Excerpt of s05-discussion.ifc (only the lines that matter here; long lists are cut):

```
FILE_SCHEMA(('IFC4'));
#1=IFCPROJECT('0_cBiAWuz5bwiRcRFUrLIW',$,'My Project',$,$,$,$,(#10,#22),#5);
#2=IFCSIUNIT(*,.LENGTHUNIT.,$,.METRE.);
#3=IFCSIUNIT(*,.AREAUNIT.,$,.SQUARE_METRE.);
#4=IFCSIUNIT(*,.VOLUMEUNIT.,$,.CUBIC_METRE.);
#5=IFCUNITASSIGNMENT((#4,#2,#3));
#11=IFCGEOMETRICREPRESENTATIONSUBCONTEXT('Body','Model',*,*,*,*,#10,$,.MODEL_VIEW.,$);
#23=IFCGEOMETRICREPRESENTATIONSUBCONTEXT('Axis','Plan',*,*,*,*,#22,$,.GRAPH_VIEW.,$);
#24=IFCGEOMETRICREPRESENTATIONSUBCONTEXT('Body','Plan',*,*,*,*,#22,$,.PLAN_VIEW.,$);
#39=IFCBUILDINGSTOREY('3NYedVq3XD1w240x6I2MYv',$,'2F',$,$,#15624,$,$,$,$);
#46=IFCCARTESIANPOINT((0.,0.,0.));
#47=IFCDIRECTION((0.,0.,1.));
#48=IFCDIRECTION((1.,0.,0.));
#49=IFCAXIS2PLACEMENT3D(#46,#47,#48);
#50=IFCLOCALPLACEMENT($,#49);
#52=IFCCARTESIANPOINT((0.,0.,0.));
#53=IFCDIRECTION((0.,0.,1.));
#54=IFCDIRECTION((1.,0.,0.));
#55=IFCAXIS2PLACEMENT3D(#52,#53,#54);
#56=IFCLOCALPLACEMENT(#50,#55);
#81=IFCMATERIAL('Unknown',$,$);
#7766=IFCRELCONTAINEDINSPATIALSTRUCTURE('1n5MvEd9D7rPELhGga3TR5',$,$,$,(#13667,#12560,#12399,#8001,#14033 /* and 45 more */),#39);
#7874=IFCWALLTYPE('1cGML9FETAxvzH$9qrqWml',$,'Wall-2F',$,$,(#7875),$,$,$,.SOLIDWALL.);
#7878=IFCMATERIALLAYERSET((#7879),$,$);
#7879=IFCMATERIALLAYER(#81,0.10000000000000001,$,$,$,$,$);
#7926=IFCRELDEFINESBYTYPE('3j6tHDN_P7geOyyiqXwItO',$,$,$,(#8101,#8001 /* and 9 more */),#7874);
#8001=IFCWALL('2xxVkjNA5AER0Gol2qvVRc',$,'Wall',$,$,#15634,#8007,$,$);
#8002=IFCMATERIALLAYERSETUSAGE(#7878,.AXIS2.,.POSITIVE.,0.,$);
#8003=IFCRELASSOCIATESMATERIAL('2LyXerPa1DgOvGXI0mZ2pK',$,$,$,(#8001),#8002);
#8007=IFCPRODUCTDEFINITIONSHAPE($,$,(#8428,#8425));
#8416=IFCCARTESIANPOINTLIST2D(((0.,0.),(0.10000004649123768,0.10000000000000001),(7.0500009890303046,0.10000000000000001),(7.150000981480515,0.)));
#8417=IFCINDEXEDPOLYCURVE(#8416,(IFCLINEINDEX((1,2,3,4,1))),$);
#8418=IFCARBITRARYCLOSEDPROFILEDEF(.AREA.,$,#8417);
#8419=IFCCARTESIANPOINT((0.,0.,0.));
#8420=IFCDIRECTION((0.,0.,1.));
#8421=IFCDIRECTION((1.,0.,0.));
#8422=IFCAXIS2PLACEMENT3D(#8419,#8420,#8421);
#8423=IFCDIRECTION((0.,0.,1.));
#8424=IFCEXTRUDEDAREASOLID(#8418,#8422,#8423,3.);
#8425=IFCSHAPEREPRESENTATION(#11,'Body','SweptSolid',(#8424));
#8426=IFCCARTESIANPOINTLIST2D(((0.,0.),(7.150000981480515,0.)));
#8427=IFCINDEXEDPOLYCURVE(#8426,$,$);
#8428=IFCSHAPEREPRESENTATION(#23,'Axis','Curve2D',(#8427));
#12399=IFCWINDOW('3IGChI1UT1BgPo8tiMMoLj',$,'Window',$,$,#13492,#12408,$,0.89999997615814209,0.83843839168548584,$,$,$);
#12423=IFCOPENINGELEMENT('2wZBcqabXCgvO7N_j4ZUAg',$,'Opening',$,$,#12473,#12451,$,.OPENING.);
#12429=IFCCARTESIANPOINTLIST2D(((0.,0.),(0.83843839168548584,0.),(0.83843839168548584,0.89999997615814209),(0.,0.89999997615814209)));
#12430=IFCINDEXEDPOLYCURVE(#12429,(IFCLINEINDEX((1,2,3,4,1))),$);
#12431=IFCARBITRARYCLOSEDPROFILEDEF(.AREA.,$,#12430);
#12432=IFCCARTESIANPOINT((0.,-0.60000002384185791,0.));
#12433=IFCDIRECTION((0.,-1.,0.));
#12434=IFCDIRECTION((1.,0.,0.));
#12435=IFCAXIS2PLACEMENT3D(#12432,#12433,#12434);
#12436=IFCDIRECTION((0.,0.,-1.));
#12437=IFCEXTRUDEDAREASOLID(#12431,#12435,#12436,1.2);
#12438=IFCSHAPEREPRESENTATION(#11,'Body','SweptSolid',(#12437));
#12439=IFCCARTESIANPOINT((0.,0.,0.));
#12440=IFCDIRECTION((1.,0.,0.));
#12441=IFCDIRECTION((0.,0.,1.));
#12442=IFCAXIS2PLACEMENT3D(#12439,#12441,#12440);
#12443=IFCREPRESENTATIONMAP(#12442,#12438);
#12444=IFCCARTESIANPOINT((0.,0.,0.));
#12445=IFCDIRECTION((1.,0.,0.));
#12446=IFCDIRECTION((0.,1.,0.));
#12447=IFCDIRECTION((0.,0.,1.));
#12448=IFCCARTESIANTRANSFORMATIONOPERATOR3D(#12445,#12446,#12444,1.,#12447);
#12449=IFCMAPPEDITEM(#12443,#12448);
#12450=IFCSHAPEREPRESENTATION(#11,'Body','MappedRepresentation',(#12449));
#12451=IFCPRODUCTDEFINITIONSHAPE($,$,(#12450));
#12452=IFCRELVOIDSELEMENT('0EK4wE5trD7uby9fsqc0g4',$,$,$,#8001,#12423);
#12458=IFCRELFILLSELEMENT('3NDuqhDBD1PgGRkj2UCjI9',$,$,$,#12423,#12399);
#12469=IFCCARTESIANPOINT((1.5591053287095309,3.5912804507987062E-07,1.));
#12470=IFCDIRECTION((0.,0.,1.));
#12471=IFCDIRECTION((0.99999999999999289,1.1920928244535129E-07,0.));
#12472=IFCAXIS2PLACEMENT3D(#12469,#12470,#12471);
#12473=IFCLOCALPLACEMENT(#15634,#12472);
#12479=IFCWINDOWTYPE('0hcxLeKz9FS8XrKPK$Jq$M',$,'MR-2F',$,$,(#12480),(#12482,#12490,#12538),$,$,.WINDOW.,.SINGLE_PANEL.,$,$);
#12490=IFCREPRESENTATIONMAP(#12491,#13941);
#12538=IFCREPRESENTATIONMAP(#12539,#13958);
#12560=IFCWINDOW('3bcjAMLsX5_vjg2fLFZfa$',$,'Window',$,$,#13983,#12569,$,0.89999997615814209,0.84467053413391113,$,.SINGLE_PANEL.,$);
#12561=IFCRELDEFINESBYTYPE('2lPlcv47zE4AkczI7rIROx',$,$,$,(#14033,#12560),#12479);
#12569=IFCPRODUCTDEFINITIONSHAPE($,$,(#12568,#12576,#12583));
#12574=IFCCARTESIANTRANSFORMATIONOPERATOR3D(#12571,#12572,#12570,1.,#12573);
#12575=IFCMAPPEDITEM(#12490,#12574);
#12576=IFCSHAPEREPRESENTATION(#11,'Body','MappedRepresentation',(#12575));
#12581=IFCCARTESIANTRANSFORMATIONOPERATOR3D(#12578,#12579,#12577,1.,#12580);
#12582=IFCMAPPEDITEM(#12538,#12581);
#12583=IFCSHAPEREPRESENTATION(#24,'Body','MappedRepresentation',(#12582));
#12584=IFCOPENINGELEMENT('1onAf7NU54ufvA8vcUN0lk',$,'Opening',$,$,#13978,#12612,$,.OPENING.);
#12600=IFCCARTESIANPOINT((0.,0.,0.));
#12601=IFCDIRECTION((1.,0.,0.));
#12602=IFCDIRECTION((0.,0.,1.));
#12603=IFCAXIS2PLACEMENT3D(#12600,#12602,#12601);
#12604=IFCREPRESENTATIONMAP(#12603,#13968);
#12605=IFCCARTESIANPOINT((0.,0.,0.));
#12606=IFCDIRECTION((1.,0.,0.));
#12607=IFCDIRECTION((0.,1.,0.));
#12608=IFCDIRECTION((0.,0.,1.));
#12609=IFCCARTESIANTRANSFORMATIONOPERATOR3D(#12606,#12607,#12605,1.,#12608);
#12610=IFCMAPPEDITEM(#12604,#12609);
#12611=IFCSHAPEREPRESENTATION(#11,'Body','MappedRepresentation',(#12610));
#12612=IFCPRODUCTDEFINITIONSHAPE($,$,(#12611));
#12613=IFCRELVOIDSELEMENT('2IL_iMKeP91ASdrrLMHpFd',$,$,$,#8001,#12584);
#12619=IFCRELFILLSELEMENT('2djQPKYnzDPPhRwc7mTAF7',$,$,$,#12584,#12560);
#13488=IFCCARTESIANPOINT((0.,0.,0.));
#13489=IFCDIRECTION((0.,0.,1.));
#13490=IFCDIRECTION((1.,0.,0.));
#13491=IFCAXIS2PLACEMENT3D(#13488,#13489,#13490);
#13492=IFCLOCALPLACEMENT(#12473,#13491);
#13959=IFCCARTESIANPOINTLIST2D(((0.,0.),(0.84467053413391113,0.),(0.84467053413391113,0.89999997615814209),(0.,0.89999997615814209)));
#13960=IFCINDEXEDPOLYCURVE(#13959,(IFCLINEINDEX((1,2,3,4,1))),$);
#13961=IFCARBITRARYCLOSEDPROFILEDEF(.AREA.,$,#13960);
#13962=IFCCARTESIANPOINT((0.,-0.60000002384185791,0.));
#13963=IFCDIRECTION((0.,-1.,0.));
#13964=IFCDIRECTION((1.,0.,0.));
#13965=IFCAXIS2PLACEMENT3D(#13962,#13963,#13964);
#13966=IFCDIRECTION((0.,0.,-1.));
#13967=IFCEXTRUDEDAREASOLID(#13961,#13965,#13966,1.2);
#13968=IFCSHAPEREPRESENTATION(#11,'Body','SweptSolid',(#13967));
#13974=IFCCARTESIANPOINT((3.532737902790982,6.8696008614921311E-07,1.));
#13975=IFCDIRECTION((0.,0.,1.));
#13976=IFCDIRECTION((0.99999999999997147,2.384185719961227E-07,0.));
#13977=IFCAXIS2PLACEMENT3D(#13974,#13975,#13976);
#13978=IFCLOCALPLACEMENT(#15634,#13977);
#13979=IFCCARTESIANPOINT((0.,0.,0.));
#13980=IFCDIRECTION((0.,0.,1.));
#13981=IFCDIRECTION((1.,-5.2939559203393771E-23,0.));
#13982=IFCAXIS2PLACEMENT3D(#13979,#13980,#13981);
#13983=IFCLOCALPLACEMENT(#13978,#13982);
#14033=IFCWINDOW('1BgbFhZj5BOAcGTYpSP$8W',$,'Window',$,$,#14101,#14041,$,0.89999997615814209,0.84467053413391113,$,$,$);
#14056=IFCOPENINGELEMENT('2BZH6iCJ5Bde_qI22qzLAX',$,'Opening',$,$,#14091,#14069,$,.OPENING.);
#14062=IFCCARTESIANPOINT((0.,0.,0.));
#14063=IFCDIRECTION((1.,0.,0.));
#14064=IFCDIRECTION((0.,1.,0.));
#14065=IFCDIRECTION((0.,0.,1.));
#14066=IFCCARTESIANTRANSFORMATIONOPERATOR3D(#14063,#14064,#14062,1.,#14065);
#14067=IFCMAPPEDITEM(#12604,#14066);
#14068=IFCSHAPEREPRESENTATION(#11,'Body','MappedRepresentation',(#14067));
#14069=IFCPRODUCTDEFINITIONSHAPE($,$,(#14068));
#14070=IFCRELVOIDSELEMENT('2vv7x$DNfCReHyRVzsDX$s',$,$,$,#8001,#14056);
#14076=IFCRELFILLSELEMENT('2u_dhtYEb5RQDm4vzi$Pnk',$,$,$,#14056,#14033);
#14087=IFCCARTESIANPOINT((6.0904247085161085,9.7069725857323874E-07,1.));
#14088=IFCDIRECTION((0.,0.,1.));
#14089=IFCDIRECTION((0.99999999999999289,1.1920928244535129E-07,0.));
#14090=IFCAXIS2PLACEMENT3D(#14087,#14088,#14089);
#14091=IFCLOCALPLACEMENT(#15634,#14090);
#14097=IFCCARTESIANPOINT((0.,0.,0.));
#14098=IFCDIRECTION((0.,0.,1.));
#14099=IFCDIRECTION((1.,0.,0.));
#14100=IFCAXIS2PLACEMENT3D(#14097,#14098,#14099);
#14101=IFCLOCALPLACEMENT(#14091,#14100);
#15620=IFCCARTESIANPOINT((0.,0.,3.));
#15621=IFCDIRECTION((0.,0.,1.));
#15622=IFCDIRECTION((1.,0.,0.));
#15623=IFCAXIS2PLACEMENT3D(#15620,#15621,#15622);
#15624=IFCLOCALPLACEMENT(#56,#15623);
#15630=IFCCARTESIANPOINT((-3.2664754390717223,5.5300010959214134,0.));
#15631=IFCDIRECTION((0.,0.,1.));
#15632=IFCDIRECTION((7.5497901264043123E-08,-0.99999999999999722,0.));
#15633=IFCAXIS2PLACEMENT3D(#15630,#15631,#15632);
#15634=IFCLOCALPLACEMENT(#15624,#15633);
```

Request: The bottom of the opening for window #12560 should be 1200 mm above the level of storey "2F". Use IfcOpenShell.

```python
import numpy as np
import ifcopenshell
import ifcopenshell.api.geometry
import ifcopenshell.geom
import ifcopenshell.util.element
import ifcopenshell.util.placement
import ifcopenshell.util.shape
import ifcopenshell.util.unit

model = ifcopenshell.open("s05-discussion.ifc")
unit_scale = ifcopenshell.util.unit.calculate_unit_scale(model)

window = model.by_guid("3bcjAMLsX5_vjg2fLFZfa$")
opening = window.FillsVoids[0].RelatingOpeningElement
storey = ifcopenshell.util.element.get_container(window, ifc_class="IfcBuildingStorey")
level = ifcopenshell.util.placement.get_local_placement(storey.ObjectPlacement)[2, 3]

# The opening's origin need not be at the sill, so measure its lowest point.
shape = ifcopenshell.geom.create_shape(ifcopenshell.geom.settings(), opening)
bottom = ifcopenshell.util.shape.get_shape_bottom_elevation(shape, shape.geometry) / unit_scale
dz = level + 1.2 / unit_scale - bottom

shift = np.array([0.0, 0.0, dz])
# The window is placed relative to its opening, so it follows when the opening moves.
matrix = ifcopenshell.util.placement.get_local_placement(opening.ObjectPlacement)
matrix[:3, 3] += shift
ifcopenshell.api.geometry.edit_object_placement(
    model, product=opening, matrix=matrix, is_si=False, should_transform_children=True
)

print(f"moved by {dz * unit_scale:+.3f} m")

model.write("s05-discussion_rev.ifc")
```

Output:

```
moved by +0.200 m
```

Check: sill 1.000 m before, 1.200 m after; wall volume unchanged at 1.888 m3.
